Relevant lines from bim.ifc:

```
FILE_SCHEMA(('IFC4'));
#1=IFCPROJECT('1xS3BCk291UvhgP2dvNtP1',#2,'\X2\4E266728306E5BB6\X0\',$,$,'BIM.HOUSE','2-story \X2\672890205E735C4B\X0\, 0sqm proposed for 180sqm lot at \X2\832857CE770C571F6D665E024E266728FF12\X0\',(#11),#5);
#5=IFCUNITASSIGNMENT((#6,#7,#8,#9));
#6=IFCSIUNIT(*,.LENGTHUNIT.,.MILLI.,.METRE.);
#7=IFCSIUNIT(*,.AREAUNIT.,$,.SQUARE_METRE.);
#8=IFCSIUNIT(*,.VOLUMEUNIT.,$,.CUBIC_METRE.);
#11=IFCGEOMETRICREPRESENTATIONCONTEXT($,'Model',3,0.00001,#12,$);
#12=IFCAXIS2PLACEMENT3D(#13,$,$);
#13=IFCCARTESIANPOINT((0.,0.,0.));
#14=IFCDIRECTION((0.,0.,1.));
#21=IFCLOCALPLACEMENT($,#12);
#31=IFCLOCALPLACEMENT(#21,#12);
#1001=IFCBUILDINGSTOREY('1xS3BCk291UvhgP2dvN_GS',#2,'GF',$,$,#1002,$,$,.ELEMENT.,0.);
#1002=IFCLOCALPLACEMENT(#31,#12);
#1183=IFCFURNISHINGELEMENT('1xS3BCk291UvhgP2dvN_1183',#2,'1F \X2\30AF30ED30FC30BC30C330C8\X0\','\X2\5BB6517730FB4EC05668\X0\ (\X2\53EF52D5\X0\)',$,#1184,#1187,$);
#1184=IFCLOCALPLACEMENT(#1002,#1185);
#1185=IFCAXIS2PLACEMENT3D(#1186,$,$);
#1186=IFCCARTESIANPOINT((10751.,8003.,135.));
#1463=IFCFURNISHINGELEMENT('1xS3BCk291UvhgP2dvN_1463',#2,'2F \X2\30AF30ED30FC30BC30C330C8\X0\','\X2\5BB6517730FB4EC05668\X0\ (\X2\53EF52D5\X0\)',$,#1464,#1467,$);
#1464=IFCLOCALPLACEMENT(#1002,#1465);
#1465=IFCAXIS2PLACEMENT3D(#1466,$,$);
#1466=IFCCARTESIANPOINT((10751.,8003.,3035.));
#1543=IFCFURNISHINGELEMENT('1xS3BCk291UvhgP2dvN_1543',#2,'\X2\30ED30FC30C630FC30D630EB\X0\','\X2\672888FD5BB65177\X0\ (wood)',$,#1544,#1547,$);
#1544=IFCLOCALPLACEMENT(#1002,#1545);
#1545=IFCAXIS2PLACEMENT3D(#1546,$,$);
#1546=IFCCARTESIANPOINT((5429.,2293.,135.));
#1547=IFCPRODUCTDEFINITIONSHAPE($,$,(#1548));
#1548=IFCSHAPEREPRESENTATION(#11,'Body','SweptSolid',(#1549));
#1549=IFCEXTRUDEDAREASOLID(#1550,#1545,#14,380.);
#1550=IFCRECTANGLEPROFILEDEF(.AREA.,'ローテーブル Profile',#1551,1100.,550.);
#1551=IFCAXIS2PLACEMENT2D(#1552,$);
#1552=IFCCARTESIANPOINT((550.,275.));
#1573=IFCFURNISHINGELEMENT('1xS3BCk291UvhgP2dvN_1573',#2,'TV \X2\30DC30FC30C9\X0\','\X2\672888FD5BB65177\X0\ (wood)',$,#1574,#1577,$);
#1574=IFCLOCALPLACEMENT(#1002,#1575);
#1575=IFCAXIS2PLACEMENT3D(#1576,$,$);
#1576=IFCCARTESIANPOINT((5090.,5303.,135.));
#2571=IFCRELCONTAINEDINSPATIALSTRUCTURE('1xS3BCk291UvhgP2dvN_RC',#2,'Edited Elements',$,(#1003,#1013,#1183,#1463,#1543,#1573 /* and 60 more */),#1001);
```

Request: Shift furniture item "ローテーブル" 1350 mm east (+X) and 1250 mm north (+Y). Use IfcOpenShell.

```python
import ifcopenshell
import ifcopenshell.api.geometry
import ifcopenshell.util.placement

model = ifcopenshell.open("bim.ifc")

item = model.by_guid("1xS3BCk291UvhgP2dvN_1543")
matrix = ifcopenshell.util.placement.get_local_placement(item.ObjectPlacement)
matrix[0, 3] += 1350.0
matrix[1, 3] += 1250.0
ifcopenshell.api.geometry.edit_object_placement(model, product=item, matrix=matrix, is_si=False)

print(ifcopenshell.util.placement.get_local_placement(item.ObjectPlacement).round(3) + 0.0)

model.write("bim_edited.ifc")
```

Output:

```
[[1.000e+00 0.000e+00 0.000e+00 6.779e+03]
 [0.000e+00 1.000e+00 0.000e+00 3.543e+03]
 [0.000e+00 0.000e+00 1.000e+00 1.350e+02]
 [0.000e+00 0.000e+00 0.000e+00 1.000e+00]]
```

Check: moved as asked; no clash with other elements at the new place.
